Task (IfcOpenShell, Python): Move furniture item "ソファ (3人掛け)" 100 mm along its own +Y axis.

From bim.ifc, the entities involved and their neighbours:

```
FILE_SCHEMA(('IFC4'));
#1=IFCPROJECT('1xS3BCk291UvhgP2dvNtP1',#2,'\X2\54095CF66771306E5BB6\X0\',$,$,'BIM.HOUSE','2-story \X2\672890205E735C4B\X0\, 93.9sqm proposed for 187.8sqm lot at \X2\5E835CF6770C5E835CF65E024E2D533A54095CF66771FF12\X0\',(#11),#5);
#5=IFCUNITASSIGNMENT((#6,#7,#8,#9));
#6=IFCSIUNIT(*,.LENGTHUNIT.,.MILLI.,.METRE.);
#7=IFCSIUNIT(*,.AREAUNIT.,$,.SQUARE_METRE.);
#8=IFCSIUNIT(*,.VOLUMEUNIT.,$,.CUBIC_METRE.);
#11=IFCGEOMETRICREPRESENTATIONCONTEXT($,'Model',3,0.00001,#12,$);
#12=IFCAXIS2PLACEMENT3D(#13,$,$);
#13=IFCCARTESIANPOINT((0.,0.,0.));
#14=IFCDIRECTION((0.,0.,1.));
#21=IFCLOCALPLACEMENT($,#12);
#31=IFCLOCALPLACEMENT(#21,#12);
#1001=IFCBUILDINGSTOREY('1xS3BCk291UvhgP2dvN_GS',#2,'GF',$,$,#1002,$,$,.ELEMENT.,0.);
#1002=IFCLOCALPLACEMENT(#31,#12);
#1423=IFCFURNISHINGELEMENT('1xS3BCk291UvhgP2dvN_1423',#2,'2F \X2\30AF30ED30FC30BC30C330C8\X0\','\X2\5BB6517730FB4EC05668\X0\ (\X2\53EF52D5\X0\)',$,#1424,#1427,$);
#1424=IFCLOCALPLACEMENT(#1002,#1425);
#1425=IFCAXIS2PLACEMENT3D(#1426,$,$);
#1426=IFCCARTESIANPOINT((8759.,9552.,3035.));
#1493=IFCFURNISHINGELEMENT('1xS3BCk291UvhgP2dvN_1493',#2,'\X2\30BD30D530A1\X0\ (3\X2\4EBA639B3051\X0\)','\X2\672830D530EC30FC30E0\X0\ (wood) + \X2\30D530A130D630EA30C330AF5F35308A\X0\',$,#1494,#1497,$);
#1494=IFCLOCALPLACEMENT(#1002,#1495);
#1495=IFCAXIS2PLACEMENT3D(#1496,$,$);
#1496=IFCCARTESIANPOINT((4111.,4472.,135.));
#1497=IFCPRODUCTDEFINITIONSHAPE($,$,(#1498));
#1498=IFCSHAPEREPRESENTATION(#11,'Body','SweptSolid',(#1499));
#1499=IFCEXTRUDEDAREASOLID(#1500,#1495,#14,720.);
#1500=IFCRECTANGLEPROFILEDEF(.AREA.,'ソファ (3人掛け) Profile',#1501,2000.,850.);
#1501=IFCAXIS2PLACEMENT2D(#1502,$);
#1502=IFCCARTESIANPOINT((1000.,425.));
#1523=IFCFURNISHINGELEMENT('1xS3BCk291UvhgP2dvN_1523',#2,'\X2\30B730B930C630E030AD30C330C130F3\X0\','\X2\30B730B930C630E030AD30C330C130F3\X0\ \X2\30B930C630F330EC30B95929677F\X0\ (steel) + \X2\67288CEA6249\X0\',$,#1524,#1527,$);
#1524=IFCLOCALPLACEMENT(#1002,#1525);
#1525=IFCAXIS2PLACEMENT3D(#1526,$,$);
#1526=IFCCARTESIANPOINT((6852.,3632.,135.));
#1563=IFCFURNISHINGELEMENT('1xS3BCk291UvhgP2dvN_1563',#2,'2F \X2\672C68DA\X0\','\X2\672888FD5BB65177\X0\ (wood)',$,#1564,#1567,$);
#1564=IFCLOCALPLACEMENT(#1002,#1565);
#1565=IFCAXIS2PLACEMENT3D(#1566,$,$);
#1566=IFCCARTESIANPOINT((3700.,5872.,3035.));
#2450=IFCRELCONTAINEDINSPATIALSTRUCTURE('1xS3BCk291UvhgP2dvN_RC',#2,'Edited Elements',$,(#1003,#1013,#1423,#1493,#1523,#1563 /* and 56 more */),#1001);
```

```python
import ifcopenshell
import ifcopenshell.api.geometry
import ifcopenshell.util.placement
import ifcopenshell.util.unit

model = ifcopenshell.open("bim.ifc")
unit_scale = ifcopenshell.util.unit.calculate_unit_scale(model)

item = model.by_guid("1xS3BCk291UvhgP2dvN_1493")
matrix = ifcopenshell.util.placement.get_local_placement(item.ObjectPlacement)
matrix[:3, 3] += matrix[:3, 1] * 0.1 / unit_scale
ifcopenshell.api.geometry.edit_object_placement(model, product=item, matrix=matrix, is_si=False)

print(ifcopenshell.util.placement.get_local_placement(item.ObjectPlacement).round(3) + 0.0)

model.write("bim_rev.ifc")
```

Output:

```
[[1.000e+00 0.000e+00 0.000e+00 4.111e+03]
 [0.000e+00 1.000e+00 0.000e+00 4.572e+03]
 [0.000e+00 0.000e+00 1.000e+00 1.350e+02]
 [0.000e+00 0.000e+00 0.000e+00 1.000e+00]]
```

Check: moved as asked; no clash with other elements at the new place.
